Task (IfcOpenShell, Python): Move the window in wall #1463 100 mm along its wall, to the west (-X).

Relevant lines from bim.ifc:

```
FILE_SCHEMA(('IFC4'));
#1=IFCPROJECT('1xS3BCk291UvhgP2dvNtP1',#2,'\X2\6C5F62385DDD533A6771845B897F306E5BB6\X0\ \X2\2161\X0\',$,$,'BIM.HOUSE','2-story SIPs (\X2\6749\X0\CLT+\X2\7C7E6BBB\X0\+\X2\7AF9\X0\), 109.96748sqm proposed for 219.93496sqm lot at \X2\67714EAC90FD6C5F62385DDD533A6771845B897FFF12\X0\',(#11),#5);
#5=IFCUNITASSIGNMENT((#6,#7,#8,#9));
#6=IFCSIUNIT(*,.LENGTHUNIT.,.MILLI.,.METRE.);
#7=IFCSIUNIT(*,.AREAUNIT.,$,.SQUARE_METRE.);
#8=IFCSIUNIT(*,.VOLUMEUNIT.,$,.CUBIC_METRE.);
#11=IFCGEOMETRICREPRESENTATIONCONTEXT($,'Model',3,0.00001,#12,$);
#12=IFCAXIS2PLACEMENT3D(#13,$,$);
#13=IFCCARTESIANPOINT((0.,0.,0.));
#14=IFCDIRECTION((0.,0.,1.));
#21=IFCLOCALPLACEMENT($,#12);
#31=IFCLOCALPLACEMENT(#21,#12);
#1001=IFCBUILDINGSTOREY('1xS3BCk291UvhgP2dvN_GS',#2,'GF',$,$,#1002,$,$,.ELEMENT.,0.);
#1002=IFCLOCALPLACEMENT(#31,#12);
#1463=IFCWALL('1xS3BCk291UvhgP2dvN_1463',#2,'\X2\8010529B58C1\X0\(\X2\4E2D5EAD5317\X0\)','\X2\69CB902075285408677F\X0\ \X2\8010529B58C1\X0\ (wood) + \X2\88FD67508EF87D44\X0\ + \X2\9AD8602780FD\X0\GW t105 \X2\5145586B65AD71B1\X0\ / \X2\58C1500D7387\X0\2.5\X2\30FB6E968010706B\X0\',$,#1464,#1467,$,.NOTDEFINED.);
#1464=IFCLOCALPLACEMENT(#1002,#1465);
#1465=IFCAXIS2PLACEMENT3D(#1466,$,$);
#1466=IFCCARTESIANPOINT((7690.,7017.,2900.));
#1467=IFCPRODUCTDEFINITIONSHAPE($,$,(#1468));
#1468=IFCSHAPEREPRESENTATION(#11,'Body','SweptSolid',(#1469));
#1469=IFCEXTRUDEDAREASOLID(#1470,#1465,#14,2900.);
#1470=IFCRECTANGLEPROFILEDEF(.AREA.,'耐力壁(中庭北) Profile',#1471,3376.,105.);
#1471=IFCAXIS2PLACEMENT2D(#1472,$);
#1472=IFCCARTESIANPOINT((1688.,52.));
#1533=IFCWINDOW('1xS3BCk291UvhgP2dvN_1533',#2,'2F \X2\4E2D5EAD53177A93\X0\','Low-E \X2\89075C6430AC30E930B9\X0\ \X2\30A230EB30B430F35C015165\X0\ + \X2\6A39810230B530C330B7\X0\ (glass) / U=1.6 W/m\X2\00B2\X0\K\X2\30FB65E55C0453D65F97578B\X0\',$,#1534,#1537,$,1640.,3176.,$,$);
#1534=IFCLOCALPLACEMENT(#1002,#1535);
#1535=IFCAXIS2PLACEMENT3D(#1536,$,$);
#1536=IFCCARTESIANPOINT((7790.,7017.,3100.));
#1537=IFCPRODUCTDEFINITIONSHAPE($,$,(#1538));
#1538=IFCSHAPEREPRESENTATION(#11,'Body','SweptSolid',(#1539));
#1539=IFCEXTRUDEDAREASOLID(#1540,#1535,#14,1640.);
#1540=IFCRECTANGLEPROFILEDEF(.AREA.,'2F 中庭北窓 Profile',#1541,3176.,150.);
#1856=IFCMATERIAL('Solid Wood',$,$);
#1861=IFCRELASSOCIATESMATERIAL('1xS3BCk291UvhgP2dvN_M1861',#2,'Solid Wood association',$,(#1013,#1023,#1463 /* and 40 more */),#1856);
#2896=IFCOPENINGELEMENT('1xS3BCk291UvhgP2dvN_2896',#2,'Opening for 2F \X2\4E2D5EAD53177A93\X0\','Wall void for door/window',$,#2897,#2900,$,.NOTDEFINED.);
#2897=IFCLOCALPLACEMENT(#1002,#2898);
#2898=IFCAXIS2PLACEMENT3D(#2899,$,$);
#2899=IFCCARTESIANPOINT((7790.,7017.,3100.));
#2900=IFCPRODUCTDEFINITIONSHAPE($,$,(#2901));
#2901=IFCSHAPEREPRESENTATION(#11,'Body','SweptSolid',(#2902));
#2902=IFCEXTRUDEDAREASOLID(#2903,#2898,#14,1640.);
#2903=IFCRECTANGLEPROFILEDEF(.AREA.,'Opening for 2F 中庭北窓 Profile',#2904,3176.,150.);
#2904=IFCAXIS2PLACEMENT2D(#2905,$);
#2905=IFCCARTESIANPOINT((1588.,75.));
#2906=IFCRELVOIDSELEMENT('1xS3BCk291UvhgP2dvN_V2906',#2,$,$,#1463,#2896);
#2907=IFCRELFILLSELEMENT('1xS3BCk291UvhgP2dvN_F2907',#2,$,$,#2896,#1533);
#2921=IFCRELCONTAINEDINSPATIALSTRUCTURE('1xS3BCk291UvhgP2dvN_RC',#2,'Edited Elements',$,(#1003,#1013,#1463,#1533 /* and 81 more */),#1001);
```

```python
import ifcopenshell
import ifcopenshell.api.geometry
import ifcopenshell.util.placement

model = ifcopenshell.open("bim.ifc")

window = model.by_guid("1xS3BCk291UvhgP2dvN_1533")
opening = window.FillsVoids[0].RelatingOpeningElement
wall = opening.VoidsElements[0].RelatingBuildingElement

wall_matrix = ifcopenshell.util.placement.get_local_placement(wall.ObjectPlacement)
shift = wall_matrix[:3, 0] * -100.0
before = ifcopenshell.util.placement.get_local_placement(window.ObjectPlacement)[:3, 3].copy()

# The window is not placed relative to its opening, so move both.
for product in (opening, window):
    matrix = ifcopenshell.util.placement.get_local_placement(product.ObjectPlacement)
    matrix[:3, 3] += shift
    ifcopenshell.api.geometry.edit_object_placement(model, product=product, matrix=matrix, is_si=False)

after = ifcopenshell.util.placement.get_local_placement(window.ObjectPlacement)[:3, 3]
print("window moved by", (after - before).round(3) + 0.0)

model.write("bim_updated.ifc")
```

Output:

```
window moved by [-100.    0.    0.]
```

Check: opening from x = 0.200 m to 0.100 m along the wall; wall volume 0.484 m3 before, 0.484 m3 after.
